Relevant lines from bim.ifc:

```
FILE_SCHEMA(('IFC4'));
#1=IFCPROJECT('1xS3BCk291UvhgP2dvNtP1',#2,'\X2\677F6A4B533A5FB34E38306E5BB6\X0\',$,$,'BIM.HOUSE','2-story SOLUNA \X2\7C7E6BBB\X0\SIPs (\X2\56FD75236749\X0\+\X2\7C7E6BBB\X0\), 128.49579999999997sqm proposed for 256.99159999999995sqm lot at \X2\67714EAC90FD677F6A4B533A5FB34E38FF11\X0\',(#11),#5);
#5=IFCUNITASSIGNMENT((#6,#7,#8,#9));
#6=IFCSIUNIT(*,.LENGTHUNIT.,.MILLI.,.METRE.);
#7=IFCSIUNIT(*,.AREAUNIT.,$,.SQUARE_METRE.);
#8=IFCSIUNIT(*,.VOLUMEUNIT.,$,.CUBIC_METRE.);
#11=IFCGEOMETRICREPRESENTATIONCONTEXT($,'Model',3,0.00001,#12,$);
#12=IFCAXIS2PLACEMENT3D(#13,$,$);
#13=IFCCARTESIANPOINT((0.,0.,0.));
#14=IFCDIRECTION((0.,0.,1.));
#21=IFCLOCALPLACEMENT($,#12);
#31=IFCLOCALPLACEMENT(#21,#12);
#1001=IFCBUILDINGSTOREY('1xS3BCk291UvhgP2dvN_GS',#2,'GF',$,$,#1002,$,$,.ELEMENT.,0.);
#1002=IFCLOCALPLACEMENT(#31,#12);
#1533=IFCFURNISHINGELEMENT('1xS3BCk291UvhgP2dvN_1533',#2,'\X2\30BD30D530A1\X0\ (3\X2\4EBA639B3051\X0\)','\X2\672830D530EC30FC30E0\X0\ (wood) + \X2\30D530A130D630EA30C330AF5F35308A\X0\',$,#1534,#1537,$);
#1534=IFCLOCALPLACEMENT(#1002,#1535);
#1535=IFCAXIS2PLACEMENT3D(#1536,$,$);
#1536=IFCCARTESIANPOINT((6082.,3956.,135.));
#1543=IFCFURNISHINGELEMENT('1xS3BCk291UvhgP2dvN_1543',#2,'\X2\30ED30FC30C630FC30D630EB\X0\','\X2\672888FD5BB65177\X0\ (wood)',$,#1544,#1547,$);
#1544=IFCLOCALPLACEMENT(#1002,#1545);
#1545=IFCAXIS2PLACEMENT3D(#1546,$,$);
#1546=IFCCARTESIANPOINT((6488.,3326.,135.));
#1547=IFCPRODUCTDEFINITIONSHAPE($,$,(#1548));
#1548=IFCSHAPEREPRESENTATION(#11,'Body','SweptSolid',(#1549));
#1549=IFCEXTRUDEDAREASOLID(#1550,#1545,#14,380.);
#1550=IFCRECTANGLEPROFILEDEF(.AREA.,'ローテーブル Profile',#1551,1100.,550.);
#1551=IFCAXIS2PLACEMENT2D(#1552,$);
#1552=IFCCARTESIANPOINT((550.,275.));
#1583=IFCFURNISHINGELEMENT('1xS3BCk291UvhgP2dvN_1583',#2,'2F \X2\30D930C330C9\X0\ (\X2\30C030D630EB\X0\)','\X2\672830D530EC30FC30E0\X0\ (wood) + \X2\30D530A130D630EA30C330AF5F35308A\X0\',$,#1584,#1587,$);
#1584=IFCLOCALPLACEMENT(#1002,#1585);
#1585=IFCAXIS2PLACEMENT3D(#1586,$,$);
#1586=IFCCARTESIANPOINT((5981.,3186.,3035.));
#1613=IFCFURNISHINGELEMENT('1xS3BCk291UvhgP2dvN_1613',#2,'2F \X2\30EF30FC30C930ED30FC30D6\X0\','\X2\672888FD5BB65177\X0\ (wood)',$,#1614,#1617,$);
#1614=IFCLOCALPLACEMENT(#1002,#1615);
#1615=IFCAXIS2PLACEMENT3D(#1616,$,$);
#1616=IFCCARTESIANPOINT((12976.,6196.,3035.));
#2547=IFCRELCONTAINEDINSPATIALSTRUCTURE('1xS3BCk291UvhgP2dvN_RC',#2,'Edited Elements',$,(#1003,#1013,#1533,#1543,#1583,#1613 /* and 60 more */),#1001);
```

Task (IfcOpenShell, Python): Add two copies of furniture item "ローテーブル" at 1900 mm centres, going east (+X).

```python
import numpy as np
import ifcopenshell
import ifcopenshell.api.geometry
import ifcopenshell.api.root
import ifcopenshell.util.element
import ifcopenshell.util.placement

model = ifcopenshell.open("bim.ifc")


def reuse_history(source, copy):
    """copy_class also copies each property set's owner history, people and application; keep the originals."""
    for rel in copy.IsDefinedBy:
        if rel.is_a("IfcRelDefinesByProperties") and (history := rel.RelatingPropertyDefinition.OwnerHistory):
            rel.RelatingPropertyDefinition.OwnerHistory = source.OwnerHistory
            ifcopenshell.util.element.remove_deep2(model, history)


source = model.by_guid("1xS3BCk291UvhgP2dvN_1543")
base = ifcopenshell.util.placement.get_local_placement(source.ObjectPlacement)
step = np.array([1.0, 0.0, 0.0]) * 1900.0

for i in range(1, 3):
    copy = ifcopenshell.api.root.copy_class(model, product=source)
    copy.Representation = ifcopenshell.util.element.copy_deep(
        model, source.Representation, exclude=["IfcGeometricRepresentationContext", "IfcRepresentationMap"]
    )
    reuse_history(source, copy)
    matrix = base.copy()
    matrix[:3, 3] += i * step
    print("added at", matrix[:3, 3].round(3) + 0.0)
    ifcopenshell.api.geometry.edit_object_placement(model, product=copy, matrix=matrix, is_si=False)

model.write("bim_updated.ifc")
```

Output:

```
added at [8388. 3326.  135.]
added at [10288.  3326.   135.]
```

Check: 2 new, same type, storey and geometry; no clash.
